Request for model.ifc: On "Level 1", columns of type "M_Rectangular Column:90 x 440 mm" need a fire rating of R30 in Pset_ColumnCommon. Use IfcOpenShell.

First a look at what the model holds.

```python
import ifcopenshell
import ifcopenshell.util.element

model = ifcopenshell.open("model.ifc")
print(model.schema)
storey = next(s for s in model.by_type("IfcBuildingStorey") if s.Name == "Level 1")
columns = [e for e in ifcopenshell.util.element.get_decomposition(storey) if e.is_a("IfcColumn")]
seen = {}
for e in columns:
    element_type = ifcopenshell.util.element.get_type(e)
    key = (element_type.Name if element_type != e and element_type else None, ifcopenshell.util.element.get_pset(e, "Pset_ColumnCommon", "FireRating"))
    seen[key] = seen.get(key, 0) + 1
for (name, value), count in sorted(seen.items(), key=str):
    print(count, "x", name, "|", value)
```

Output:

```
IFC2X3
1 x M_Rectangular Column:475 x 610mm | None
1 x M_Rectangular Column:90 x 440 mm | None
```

```python
import ifcopenshell
import ifcopenshell.api.pset
import ifcopenshell.util.element

model = ifcopenshell.open("model.ifc")

storey = next(s for s in model.by_type("IfcBuildingStorey") if s.Name == "Level 1")
columns = [e for e in ifcopenshell.util.element.get_decomposition(storey) if e.is_a("IfcColumn")]

count = 0
for e in columns:
    element_type = ifcopenshell.util.element.get_type(e)
    if element_type in (None, e) or element_type.Name != "M_Rectangular Column:90 x 440 mm":
        continue
    # add_pset returns the element's existing set when there is one.
    pset = ifcopenshell.api.pset.add_pset(model, product=e, name="Pset_ColumnCommon")
    ifcopenshell.api.pset.edit_pset(model, pset=pset, properties={"FireRating": "R30"})
    count += 1

print(count, "columns updated")

model.write("model_updated.ifc")
```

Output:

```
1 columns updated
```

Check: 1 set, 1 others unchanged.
